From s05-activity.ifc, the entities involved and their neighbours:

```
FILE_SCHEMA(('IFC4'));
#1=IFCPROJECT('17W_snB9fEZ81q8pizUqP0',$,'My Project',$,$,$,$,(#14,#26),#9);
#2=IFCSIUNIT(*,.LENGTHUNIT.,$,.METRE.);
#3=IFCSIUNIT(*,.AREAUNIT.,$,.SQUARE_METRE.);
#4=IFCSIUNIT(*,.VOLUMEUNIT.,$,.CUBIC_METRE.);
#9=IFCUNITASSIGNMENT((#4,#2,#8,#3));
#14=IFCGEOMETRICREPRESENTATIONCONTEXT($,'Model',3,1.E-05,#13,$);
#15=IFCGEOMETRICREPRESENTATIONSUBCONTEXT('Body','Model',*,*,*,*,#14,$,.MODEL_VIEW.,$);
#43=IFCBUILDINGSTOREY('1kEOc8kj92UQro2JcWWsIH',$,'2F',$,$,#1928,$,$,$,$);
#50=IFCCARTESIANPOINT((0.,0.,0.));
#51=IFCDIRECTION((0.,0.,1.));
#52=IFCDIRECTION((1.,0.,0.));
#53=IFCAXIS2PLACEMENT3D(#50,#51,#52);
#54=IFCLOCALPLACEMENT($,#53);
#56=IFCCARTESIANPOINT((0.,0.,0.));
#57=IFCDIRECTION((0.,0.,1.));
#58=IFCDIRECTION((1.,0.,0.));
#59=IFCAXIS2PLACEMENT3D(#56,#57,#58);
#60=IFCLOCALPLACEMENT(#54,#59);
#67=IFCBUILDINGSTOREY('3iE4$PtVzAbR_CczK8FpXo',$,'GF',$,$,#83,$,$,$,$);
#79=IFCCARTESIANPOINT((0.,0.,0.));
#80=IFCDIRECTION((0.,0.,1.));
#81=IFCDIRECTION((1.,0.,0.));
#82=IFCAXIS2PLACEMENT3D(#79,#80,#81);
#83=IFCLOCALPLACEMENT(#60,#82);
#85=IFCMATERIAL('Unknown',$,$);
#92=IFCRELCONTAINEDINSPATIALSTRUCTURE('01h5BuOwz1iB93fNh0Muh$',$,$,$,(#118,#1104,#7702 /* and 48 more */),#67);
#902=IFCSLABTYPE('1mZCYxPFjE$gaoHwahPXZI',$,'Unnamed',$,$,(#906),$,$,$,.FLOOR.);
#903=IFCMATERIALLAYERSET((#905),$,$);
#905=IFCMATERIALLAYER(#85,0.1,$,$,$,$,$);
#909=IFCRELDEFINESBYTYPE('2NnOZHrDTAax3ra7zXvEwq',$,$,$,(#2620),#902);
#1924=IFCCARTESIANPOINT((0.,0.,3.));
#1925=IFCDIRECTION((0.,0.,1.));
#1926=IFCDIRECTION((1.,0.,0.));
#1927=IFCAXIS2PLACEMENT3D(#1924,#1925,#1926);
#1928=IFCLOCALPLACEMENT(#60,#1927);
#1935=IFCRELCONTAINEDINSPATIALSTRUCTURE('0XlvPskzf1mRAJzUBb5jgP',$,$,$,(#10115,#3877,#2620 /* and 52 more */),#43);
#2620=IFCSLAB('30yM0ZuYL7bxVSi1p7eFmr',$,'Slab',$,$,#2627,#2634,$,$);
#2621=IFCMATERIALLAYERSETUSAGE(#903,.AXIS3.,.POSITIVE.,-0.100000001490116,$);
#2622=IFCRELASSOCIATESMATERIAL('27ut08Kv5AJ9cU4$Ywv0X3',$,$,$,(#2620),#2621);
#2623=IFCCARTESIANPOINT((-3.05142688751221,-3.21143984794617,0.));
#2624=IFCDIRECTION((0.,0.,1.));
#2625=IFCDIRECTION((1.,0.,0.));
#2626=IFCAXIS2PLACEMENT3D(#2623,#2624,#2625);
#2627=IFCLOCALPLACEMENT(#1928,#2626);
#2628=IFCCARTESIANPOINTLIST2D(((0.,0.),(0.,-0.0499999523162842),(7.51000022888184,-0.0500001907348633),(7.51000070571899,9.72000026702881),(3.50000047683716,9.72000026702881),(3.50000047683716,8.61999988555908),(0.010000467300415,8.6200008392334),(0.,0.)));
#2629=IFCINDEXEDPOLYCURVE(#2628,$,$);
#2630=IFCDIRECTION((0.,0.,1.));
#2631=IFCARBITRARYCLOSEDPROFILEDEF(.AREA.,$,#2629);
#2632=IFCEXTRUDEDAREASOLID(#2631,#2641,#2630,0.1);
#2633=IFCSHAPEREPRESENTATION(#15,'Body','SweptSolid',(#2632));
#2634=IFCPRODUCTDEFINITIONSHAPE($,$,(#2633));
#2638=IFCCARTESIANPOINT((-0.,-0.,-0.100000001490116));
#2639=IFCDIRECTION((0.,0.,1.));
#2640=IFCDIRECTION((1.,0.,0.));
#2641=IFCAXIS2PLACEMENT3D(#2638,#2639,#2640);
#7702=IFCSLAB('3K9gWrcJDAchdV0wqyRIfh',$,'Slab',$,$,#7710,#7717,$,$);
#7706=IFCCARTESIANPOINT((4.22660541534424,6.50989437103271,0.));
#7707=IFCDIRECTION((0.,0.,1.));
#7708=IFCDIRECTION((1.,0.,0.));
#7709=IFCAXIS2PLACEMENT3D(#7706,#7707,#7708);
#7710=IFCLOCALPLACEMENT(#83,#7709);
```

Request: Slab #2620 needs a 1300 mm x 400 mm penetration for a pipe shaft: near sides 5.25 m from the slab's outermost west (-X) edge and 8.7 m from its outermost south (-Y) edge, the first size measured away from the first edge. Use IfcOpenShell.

```python
import numpy as np
import ifcopenshell
import ifcopenshell.api.feature
import ifcopenshell.api.geometry
import ifcopenshell.api.root
import ifcopenshell.geom
import ifcopenshell.util.placement
import ifcopenshell.util.representation
import ifcopenshell.util.shape
import ifcopenshell.util.unit

model = ifcopenshell.open("s05-activity.ifc")
unit_scale = ifcopenshell.util.unit.calculate_unit_scale(model)
settings = ifcopenshell.geom.settings()


def volume(element):
    """Net volume in cubic metres, openings subtracted."""
    shape = ifcopenshell.geom.create_shape(settings, element)
    return ifcopenshell.util.shape.get_volume(shape.geometry)


slab = model.by_guid("30yM0ZuYL7bxVSi1p7eFmr")
before = volume(slab)

# Extent in the slab's own axes, in metres. The edges named are its -X and -Y sides.
slab_shape = ifcopenshell.geom.create_shape(settings, slab)
vertices = ifcopenshell.util.shape.get_vertices(slab_shape.geometry)
x_min, y_min, bottom = vertices.min(axis=0)
top = vertices[:, 2].max()

opening = ifcopenshell.api.root.create_entity(model, ifc_class="IfcOpeningElement", name="Pipe shaft opening", predefined_type="OPENING")
context = ifcopenshell.util.representation.get_context(model, "Model", "Body", "MODEL_VIEW")
width, depth = 1.3, 0.4
outline = [(0.0, 0.0), (width, 0.0), (width, depth), (0.0, depth), (0.0, 0.0)]
# Overshoot both faces by 50 mm so the cut is clean.
shape = ifcopenshell.api.geometry.add_slab_representation(
    model, context=context, depth=top - bottom + 0.1, polyline=outline
)
ifcopenshell.api.geometry.assign_representation(model, product=opening, representation=shape)

matrix = ifcopenshell.util.placement.get_local_placement(slab.ObjectPlacement)
matrix[:, 3] = matrix @ np.append(np.array([x_min + 5.25, y_min + 8.7, bottom - 0.05]) / unit_scale, 1.0)
ifcopenshell.api.geometry.edit_object_placement(model, product=opening, matrix=matrix, is_si=False)
ifcopenshell.api.feature.add_feature(model, feature=opening, element=slab)

after = volume(slab)

print(f"slab volume {before:.3f} -> {after:.3f} m3")

model.write("s05-activity_updated.ifc")
```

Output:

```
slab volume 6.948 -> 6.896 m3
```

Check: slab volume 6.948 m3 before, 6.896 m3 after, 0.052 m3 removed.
